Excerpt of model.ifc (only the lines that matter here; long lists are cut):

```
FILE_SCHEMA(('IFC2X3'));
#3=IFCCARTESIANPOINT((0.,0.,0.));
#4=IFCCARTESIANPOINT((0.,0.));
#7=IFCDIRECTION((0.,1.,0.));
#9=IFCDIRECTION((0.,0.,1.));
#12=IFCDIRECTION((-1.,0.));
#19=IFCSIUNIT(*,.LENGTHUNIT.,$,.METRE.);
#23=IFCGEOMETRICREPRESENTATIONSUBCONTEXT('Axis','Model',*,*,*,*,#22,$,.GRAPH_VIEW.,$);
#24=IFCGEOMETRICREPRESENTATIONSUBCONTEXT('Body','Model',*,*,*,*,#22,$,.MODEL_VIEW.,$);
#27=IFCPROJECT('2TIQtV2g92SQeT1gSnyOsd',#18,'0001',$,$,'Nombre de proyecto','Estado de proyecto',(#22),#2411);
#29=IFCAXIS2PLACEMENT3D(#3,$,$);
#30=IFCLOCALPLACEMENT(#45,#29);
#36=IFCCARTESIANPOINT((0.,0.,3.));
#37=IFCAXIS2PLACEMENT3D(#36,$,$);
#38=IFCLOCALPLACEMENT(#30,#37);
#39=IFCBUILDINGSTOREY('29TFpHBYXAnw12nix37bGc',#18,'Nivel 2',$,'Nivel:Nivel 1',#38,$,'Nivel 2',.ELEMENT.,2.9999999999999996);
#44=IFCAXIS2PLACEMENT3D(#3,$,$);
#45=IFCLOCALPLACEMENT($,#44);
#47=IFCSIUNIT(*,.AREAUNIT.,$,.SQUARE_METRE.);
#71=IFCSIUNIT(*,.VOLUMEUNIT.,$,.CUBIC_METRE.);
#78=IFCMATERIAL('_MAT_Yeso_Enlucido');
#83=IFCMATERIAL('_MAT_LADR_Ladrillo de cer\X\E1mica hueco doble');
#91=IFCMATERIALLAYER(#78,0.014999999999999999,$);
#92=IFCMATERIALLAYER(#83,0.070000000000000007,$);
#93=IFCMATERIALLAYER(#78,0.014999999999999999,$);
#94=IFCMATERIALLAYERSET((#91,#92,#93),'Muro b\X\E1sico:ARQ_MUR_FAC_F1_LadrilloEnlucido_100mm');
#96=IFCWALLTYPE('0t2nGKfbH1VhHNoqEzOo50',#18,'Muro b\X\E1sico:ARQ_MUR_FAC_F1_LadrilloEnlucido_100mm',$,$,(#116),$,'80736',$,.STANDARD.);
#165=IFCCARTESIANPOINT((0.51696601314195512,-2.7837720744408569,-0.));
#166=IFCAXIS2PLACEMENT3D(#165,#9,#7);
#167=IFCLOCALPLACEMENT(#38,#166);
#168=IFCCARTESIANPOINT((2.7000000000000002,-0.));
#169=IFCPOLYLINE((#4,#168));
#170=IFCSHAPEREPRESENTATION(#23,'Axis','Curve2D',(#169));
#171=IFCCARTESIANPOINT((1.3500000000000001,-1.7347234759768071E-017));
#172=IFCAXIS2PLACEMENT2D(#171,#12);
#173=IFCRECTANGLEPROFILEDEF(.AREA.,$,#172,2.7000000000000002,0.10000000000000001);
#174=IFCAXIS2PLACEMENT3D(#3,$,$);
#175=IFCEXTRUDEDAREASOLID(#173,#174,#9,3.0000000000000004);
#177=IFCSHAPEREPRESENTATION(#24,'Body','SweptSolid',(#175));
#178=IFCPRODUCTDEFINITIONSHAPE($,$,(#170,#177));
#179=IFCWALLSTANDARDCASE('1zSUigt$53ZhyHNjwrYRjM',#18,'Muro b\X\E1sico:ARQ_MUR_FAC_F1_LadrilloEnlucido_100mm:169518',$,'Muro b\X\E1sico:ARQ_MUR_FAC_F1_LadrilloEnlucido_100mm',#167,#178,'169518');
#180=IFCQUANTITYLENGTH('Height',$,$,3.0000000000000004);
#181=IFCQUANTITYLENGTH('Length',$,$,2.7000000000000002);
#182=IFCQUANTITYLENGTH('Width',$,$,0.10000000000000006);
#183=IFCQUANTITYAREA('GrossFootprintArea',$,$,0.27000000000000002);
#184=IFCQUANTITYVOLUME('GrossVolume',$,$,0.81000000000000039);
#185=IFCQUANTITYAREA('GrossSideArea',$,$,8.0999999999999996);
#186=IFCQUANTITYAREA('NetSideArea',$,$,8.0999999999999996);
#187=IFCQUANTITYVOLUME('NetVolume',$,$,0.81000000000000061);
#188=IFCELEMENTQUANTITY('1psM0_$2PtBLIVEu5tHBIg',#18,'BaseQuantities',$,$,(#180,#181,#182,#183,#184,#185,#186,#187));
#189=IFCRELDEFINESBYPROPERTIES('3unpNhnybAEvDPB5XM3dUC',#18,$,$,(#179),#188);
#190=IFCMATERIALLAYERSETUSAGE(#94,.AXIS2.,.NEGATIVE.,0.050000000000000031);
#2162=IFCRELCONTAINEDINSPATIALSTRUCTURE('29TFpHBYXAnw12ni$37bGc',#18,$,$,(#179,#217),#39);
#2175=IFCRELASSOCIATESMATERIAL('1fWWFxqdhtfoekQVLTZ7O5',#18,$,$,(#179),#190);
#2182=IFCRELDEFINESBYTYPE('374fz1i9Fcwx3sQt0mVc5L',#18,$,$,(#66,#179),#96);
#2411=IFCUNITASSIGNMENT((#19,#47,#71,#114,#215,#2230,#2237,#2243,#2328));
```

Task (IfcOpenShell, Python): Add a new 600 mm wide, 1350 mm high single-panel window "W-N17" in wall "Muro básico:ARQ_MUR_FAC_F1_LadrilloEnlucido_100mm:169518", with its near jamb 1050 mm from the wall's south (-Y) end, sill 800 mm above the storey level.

```python
import numpy as np
import ifcopenshell
import ifcopenshell.api.feature
import ifcopenshell.api.geometry
import ifcopenshell.api.pset
import ifcopenshell.api.root
import ifcopenshell.api.spatial
import ifcopenshell.api.type
import ifcopenshell.geom
import ifcopenshell.util.element
import ifcopenshell.util.placement
import ifcopenshell.util.representation
import ifcopenshell.util.shape
import ifcopenshell.util.unit

model = ifcopenshell.open("model.ifc")
unit_scale = ifcopenshell.util.unit.calculate_unit_scale(model)
area_scale = ifcopenshell.util.unit.calculate_unit_scale(model, "AREAUNIT")
volume_scale = ifcopenshell.util.unit.calculate_unit_scale(model, "VOLUMEUNIT")
settings = ifcopenshell.geom.settings()


def volume(element):
    """Net volume in cubic metres, openings subtracted."""
    shape = ifcopenshell.geom.create_shape(settings, element)
    return ifcopenshell.util.shape.get_volume(shape.geometry)


wall = model.by_id(179)
storey = ifcopenshell.util.element.get_container(wall, ifc_class="IfcBuildingStorey")
context = ifcopenshell.util.representation.get_context(model, "Model", "Body", "MODEL_VIEW")
before = volume(wall)

width, height, from_end, sill = 0.6, 1.35, 1.05, 0.8  # metres

# The wall runs along its own X axis, and the end named is its -X end.
wall_shape = ifcopenshell.geom.create_shape(settings, wall)
x, y, z = ifcopenshell.util.shape.get_vertices(wall_shape.geometry).T
start = x.min() + from_end
face, thickness = float(y.min()), float(y.max() - y.min())
wall_matrix = ifcopenshell.util.placement.get_local_placement(wall.ObjectPlacement)
level = ifcopenshell.util.placement.get_local_placement(storey.ObjectPlacement)[2, 3]


def in_wall(x, y):
    """Placement at x, y metres in the wall's axes, at sill height."""
    matrix = wall_matrix.copy()
    matrix[:, 3] = wall_matrix @ np.array([x / unit_scale, y / unit_scale, 0.0, 1.0])
    matrix[2, 3] = level + sill / unit_scale
    return matrix


# Opening: a box that overshoots both wall faces by 50 mm.
opening = ifcopenshell.api.root.create_entity(model, ifc_class="IfcOpeningElement")
box = ifcopenshell.api.geometry.add_wall_representation(
    model, context=context, length=width, height=height, thickness=thickness + 0.1
)
ifcopenshell.api.geometry.assign_representation(model, product=opening, representation=box)
ifcopenshell.api.geometry.edit_object_placement(model, product=opening, matrix=in_wall(start, face - 0.05), is_si=False)
ifcopenshell.api.feature.add_feature(model, feature=opening, element=wall)

window = ifcopenshell.api.root.create_entity(model, ifc_class="IfcWindow", name="W-N17")
window.OverallWidth, window.OverallHeight = width / unit_scale, height / unit_scale
body = ifcopenshell.api.geometry.add_window_representation(
    model,
    context=context,
    overall_width=window.OverallWidth,
    overall_height=window.OverallHeight,
    partition_type="SINGLE_PANEL",
)
ifcopenshell.api.geometry.assign_representation(model, product=window, representation=body)
ifcopenshell.api.spatial.assign_container(model, products=[window], relating_structure=storey)
fills = ifcopenshell.api.feature.add_filling(model, opening=opening, element=window)
fills.OwnerHistory = window.OwnerHistory  # required in IFC2X3

# IFC2X3 keeps the operation on the window style.
style = ifcopenshell.api.root.create_entity(model, ifc_class="IfcWindowStyle", name="W-N17")
style.OperationType, style.ConstructionType = "SINGLE_PANEL", "NOTDEFINED"
style.ParameterTakesPrecedence = style.Sizeable = False
ifcopenshell.api.type.assign_type(model, related_objects=[window], relating_type=style)

# Centre the window in the wall's thickness.
ifcopenshell.api.geometry.edit_object_placement(model, product=window, matrix=in_wall(start, face), is_si=False)
window_shape = ifcopenshell.geom.create_shape(settings, window)
depth = ifcopenshell.util.shape.get_vertices(window_shape.geometry)[:, 1]
offset = face + thickness / 2 - (depth.min() + depth.max()) / 2
ifcopenshell.api.geometry.edit_object_placement(model, product=window, matrix=in_wall(start, offset), is_si=False)

after = volume(wall)

# Update the wall's stored quantities.
qto = model.by_id(ifcopenshell.util.element.get_pset(wall, "BaseQuantities", should_inherit=False)["id"])
ifcopenshell.api.pset.edit_qto(model, qto=qto, properties={
    "NetSideArea": after / thickness / area_scale,
    "NetVolume": after / volume_scale,
})

print(f"wall volume {before:.3f} -> {after:.3f} m3")

model.write("model-out.ifc")
```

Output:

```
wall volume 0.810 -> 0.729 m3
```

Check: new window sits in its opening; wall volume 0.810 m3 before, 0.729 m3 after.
